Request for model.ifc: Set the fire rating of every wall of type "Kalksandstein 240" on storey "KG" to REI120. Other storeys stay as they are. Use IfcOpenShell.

First a look at what the model holds.

```python
import ifcopenshell
import ifcopenshell.util.element

model = ifcopenshell.open("model.ifc")
print(model.schema)
storey = next(s for s in model.by_type("IfcBuildingStorey") if s.Name == "KG")
walls = [e for e in ifcopenshell.util.element.get_decomposition(storey) if e.is_a("IfcWall")]
seen = {}
for e in walls:
    element_type = ifcopenshell.util.element.get_type(e)
    key = (element_type.Name if element_type != e and element_type else None, ifcopenshell.util.element.get_pset(e, "Pset_WallCommon", "FireRating"))
    seen[key] = seen.get(key, 0) + 1
for (name, value), count in sorted(seen.items(), key=str):
    print(count, "x", name, "|", value)
```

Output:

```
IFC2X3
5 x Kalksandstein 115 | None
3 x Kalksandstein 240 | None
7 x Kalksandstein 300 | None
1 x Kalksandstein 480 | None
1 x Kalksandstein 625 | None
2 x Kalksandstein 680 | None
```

```python
import ifcopenshell
import ifcopenshell.api.pset
import ifcopenshell.util.element

model = ifcopenshell.open("model.ifc")

storey = next(s for s in model.by_type("IfcBuildingStorey") if s.Name == "KG")
walls = [e for e in ifcopenshell.util.element.get_decomposition(storey) if e.is_a("IfcWall")]

count = 0
for e in walls:
    element_type = ifcopenshell.util.element.get_type(e)
    if element_type in (None, e) or element_type.Name != "Kalksandstein 240":
        continue
    # add_pset returns the element's existing set when there is one.
    pset = ifcopenshell.api.pset.add_pset(model, product=e, name="Pset_WallCommon")
    ifcopenshell.api.pset.edit_pset(model, pset=pset, properties={"FireRating": "REI120"})
    count += 1

print(count, "walls updated")

model.write("model_v2.ifc")
```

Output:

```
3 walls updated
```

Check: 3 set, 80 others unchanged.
